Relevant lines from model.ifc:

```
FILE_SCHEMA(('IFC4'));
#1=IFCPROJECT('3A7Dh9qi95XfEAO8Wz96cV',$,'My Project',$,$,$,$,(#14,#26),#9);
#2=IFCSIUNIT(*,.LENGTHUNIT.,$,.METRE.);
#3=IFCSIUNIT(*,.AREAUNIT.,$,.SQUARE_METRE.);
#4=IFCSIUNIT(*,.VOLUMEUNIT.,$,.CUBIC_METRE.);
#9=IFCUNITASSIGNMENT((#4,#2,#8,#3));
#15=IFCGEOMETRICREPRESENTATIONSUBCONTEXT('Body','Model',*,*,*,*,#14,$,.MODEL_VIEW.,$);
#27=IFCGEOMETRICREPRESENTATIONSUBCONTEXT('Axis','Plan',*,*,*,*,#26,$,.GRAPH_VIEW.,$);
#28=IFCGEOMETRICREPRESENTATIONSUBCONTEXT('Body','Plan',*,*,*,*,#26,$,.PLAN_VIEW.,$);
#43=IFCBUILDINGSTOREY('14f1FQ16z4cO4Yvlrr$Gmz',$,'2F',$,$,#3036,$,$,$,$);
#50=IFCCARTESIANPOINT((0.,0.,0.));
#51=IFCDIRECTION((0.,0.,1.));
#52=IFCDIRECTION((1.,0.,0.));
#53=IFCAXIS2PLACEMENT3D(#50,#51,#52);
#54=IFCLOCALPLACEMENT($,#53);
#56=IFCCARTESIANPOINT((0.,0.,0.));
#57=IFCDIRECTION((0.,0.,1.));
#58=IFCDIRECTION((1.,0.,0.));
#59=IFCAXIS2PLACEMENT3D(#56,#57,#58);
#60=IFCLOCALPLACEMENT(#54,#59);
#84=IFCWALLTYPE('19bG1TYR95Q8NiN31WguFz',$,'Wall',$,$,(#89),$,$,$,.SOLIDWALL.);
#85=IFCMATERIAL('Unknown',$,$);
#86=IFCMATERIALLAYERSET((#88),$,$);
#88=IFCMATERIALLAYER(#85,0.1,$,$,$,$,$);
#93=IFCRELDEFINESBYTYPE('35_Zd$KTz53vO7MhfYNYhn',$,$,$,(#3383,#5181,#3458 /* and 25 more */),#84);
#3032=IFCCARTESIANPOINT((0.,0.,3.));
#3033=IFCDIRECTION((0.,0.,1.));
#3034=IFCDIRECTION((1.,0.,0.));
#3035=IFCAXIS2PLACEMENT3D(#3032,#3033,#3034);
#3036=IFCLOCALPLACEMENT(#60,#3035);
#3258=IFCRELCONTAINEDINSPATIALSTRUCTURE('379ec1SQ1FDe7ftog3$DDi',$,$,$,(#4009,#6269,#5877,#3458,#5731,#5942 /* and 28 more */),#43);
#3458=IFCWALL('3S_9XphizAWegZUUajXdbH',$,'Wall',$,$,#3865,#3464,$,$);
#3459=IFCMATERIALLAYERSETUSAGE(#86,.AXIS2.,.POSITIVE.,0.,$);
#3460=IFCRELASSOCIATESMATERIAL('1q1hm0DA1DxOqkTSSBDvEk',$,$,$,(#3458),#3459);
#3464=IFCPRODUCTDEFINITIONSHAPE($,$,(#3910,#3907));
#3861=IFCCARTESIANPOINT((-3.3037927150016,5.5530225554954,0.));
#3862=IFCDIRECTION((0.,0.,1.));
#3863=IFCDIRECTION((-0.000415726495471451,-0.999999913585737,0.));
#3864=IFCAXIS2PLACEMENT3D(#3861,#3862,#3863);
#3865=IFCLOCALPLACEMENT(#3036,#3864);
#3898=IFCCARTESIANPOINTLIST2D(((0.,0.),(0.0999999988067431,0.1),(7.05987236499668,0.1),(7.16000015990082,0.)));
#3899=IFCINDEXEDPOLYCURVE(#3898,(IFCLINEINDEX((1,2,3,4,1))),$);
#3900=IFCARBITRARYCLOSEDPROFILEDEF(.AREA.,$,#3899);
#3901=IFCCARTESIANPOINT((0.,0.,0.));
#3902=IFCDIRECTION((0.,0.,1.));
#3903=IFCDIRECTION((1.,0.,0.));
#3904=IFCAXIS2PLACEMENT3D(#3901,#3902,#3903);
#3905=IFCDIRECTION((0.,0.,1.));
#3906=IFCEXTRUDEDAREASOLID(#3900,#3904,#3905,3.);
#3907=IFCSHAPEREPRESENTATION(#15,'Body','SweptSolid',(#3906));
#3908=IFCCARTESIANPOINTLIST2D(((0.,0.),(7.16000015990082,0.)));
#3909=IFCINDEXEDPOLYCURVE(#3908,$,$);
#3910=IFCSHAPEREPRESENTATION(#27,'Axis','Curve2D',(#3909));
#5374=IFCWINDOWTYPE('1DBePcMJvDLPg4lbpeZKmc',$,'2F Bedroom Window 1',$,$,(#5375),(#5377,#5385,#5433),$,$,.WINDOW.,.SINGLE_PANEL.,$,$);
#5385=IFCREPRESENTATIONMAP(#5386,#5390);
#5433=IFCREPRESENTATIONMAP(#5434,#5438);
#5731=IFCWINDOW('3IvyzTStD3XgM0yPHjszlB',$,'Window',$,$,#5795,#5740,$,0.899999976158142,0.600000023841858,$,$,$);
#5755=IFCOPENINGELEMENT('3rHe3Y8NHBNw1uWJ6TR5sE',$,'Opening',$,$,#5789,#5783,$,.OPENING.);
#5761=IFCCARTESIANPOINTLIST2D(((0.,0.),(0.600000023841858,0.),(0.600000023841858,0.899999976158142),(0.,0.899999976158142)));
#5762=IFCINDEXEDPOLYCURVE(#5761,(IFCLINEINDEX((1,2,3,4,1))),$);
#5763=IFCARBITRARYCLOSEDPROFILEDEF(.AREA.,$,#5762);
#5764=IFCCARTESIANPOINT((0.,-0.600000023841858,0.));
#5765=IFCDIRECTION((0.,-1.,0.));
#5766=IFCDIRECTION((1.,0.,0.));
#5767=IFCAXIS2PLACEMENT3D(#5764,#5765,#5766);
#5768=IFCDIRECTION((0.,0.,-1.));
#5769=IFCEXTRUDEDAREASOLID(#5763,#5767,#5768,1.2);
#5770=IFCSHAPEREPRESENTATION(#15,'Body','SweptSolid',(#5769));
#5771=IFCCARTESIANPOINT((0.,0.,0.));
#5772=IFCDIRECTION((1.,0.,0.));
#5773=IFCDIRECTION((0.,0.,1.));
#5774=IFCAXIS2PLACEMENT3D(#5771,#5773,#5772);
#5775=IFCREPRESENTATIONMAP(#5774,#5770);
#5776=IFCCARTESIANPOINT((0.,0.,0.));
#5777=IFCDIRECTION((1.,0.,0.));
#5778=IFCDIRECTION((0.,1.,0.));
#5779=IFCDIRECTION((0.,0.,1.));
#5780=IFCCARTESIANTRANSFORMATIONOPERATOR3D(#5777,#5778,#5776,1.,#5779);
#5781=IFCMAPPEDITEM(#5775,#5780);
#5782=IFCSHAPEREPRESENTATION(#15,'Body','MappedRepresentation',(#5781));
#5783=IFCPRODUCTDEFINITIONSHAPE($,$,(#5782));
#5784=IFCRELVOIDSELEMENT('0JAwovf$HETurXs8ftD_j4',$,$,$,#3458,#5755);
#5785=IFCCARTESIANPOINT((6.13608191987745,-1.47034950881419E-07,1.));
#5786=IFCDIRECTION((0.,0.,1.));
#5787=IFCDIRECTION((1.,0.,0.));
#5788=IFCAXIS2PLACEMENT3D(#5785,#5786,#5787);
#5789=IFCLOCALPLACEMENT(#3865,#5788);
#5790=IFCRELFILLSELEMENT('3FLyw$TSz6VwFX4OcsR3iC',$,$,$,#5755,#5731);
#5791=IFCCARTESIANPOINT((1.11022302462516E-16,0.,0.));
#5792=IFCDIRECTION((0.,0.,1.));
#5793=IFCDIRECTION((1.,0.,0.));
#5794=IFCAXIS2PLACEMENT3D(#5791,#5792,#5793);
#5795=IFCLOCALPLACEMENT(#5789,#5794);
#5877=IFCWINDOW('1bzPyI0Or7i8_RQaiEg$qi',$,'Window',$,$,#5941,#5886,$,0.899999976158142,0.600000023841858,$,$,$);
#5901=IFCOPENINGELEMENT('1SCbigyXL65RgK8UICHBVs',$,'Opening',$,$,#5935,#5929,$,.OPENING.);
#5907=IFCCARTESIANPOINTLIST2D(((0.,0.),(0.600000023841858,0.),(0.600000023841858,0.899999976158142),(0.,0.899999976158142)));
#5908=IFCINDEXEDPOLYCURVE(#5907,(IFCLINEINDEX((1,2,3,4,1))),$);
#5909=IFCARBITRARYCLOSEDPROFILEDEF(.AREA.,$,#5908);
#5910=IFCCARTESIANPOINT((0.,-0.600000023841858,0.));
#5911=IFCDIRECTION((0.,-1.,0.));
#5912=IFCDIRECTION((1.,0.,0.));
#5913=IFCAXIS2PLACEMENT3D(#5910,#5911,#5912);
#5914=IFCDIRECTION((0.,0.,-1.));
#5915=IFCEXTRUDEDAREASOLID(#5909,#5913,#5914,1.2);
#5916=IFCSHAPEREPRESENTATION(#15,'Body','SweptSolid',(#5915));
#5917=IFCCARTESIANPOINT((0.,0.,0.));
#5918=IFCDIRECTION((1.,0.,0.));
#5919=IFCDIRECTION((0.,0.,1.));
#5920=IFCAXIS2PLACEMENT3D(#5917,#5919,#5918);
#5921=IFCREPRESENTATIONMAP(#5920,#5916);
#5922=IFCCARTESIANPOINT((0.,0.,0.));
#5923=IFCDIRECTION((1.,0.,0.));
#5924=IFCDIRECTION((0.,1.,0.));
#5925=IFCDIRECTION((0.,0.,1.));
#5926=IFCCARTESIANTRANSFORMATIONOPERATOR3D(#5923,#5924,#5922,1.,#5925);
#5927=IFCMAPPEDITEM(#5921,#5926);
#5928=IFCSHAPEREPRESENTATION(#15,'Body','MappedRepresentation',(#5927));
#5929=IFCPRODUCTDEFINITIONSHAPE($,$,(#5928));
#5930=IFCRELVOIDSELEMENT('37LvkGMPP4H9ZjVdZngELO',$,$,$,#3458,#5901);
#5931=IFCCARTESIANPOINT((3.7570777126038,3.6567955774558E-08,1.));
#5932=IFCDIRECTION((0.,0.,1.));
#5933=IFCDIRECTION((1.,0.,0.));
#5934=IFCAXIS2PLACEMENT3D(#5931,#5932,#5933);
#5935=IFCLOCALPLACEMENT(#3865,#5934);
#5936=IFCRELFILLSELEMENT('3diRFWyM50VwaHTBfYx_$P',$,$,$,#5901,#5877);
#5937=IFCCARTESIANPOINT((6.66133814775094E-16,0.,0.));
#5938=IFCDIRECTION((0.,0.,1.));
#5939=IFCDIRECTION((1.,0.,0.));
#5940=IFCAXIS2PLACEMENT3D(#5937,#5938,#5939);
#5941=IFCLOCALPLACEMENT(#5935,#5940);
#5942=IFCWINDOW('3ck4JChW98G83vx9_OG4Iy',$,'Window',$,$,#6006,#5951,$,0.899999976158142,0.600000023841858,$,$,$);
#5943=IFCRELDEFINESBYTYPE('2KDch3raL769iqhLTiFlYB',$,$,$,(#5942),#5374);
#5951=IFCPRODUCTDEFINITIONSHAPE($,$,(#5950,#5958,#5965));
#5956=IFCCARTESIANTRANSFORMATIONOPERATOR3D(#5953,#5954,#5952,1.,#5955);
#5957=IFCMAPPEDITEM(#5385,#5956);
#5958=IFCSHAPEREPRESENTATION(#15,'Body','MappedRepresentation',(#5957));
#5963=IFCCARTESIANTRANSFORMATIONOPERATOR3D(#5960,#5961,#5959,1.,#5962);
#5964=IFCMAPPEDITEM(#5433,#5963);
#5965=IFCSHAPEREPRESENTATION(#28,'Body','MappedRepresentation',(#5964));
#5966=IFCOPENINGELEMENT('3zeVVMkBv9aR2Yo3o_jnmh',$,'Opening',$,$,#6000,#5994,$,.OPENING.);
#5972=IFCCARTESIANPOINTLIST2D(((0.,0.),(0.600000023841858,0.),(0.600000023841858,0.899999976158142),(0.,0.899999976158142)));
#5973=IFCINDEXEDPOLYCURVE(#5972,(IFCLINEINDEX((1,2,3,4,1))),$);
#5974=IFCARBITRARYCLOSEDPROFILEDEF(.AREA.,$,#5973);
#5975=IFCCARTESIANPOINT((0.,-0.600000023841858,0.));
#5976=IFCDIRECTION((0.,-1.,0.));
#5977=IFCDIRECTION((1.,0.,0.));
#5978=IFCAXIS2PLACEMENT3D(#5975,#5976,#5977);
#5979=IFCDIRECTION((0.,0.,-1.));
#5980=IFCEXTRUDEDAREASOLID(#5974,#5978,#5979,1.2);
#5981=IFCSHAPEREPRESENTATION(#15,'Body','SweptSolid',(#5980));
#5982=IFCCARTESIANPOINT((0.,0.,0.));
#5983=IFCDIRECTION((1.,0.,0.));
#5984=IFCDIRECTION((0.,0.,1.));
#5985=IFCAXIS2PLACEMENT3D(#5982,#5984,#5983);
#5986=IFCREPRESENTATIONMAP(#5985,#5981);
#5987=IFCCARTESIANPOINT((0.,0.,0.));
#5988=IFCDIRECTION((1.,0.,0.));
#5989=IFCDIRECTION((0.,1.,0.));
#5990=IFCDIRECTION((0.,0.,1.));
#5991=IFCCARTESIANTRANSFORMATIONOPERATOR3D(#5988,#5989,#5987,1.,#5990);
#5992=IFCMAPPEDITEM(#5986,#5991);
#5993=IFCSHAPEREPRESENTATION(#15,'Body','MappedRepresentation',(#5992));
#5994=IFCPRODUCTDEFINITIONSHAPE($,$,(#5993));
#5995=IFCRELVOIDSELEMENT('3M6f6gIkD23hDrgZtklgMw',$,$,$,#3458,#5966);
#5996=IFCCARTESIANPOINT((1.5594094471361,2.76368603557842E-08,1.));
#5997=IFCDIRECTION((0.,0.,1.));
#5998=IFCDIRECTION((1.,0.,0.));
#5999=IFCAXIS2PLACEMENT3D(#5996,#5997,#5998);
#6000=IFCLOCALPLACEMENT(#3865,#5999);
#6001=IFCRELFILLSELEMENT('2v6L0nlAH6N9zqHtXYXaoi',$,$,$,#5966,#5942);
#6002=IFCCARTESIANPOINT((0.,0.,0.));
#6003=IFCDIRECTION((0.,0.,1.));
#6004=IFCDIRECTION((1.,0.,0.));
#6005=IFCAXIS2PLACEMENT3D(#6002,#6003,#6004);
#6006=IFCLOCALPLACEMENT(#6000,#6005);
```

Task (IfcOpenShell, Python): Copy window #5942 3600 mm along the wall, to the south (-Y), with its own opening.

```python
import ifcopenshell
import ifcopenshell.api.feature
import ifcopenshell.api.geometry
import ifcopenshell.api.root
import ifcopenshell.geom
import ifcopenshell.util.element
import ifcopenshell.util.placement
import ifcopenshell.util.shape

model = ifcopenshell.open("model.ifc")
settings = ifcopenshell.geom.settings()


def volume(element):
    """Net volume in cubic metres, openings subtracted."""
    shape = ifcopenshell.geom.create_shape(settings, element)
    return ifcopenshell.util.shape.get_volume(shape.geometry)


window = model.by_guid("3ck4JChW98G83vx9_OG4Iy")
opening = window.FillsVoids[0].RelatingOpeningElement
wall = opening.VoidsElements[0].RelatingBuildingElement
before = volume(wall)
shift = ifcopenshell.util.placement.get_local_placement(wall.ObjectPlacement)[:3, 0] * 3.6

# copy_class copies the void relationship, type, container and properties, but no geometry.
new_opening = ifcopenshell.api.root.copy_class(model, product=opening)
new_opening.Representation = ifcopenshell.util.element.copy_deep(
    model, opening.Representation, exclude=["IfcGeometricRepresentationContext", "IfcRepresentationMap"]
)
new_window = ifcopenshell.api.root.copy_class(model, product=window)
new_window.Representation = ifcopenshell.util.element.copy_deep(
    model, window.Representation, exclude=["IfcGeometricRepresentationContext", "IfcRepresentationMap"]
)
ifcopenshell.api.feature.add_filling(model, opening=new_opening, element=new_window)

for old, new in ((opening, new_opening), (window, new_window)):
    matrix = ifcopenshell.util.placement.get_local_placement(old.ObjectPlacement)
    matrix[:3, 3] += shift
    ifcopenshell.api.geometry.edit_object_placement(model, product=new, matrix=matrix, is_si=False)

after = volume(wall)

print(f"wall volume {before:.3f} -> {after:.3f} m3")

model.write("model_updated.ifc")
```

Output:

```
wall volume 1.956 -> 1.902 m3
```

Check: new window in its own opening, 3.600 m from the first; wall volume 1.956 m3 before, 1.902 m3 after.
